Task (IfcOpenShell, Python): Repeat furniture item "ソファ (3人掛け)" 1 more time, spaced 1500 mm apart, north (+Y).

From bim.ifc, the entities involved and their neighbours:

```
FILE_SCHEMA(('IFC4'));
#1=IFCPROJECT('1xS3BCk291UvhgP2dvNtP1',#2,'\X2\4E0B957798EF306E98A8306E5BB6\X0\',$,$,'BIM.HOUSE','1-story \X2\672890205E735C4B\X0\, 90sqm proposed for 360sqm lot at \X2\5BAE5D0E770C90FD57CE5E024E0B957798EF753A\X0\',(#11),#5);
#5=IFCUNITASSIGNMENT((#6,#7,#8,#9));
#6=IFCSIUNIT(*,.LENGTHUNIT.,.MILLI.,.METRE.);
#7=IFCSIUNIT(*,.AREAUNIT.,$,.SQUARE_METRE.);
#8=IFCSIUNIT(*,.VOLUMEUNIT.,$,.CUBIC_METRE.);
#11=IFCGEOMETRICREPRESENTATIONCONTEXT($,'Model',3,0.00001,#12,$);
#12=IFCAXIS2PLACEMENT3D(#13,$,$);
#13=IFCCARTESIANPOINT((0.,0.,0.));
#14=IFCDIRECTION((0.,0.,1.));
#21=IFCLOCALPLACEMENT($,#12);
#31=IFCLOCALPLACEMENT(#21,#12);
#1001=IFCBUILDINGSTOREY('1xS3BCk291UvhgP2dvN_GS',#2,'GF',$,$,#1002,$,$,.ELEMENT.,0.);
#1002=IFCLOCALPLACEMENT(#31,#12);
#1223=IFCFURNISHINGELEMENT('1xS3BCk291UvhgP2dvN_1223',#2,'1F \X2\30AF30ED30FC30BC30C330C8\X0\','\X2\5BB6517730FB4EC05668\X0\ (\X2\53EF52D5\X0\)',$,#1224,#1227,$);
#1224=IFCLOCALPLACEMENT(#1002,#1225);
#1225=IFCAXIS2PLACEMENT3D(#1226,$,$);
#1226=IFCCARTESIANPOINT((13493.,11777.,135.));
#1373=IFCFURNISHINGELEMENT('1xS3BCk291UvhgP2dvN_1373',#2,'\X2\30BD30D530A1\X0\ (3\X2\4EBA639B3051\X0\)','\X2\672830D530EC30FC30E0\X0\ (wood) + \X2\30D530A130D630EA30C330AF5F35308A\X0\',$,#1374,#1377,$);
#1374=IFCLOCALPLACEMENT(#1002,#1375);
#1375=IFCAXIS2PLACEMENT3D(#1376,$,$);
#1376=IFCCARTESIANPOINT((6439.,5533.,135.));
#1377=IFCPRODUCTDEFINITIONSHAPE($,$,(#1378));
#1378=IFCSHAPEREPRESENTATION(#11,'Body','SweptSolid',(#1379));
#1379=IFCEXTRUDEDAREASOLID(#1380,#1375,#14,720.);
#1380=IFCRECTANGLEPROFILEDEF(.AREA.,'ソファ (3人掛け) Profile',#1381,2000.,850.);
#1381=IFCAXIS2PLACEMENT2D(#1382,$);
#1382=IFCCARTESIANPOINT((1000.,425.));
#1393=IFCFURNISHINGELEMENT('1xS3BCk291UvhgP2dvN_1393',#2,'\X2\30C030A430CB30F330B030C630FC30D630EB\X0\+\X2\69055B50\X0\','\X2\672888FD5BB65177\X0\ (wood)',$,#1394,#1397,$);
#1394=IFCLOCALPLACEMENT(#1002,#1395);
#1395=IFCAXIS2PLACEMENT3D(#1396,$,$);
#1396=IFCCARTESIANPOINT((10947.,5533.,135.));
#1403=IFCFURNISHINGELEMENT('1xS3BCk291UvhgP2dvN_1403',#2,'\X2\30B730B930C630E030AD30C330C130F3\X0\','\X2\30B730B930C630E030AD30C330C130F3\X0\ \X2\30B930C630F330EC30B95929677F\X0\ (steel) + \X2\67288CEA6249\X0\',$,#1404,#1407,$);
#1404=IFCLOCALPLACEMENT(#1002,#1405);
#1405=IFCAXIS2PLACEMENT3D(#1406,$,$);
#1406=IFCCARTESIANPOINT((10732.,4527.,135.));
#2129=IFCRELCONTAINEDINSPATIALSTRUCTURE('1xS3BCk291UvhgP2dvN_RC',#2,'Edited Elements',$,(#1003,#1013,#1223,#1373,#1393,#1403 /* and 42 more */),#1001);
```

```python
import numpy as np
import ifcopenshell
import ifcopenshell.api.geometry
import ifcopenshell.api.root
import ifcopenshell.util.element
import ifcopenshell.util.placement
import ifcopenshell.util.unit

model = ifcopenshell.open("bim.ifc")
unit_scale = ifcopenshell.util.unit.calculate_unit_scale(model)


def reuse_history(source, copy):
    """copy_class also copies each property set's owner history, people and application; keep the originals."""
    for rel in copy.IsDefinedBy:
        if rel.is_a("IfcRelDefinesByProperties") and (history := rel.RelatingPropertyDefinition.OwnerHistory):
            rel.RelatingPropertyDefinition.OwnerHistory = source.OwnerHistory
            ifcopenshell.util.element.remove_deep2(model, history)


source = model.by_id(1373)
base = ifcopenshell.util.placement.get_local_placement(source.ObjectPlacement)
step = np.array([0.0, 1.0, 0.0]) * 1.5 / unit_scale

for i in range(1, 2):
    copy = ifcopenshell.api.root.copy_class(model, product=source)
    copy.Representation = ifcopenshell.util.element.copy_deep(
        model, source.Representation, exclude=["IfcGeometricRepresentationContext", "IfcRepresentationMap"]
    )
    reuse_history(source, copy)
    matrix = base.copy()
    matrix[:3, 3] += i * step
    print("added at", matrix[:3, 3].round(3) + 0.0)
    ifcopenshell.api.geometry.edit_object_placement(model, product=copy, matrix=matrix, is_si=False)

model.write("bim_rev.ifc")
```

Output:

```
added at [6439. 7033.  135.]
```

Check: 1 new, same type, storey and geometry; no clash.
